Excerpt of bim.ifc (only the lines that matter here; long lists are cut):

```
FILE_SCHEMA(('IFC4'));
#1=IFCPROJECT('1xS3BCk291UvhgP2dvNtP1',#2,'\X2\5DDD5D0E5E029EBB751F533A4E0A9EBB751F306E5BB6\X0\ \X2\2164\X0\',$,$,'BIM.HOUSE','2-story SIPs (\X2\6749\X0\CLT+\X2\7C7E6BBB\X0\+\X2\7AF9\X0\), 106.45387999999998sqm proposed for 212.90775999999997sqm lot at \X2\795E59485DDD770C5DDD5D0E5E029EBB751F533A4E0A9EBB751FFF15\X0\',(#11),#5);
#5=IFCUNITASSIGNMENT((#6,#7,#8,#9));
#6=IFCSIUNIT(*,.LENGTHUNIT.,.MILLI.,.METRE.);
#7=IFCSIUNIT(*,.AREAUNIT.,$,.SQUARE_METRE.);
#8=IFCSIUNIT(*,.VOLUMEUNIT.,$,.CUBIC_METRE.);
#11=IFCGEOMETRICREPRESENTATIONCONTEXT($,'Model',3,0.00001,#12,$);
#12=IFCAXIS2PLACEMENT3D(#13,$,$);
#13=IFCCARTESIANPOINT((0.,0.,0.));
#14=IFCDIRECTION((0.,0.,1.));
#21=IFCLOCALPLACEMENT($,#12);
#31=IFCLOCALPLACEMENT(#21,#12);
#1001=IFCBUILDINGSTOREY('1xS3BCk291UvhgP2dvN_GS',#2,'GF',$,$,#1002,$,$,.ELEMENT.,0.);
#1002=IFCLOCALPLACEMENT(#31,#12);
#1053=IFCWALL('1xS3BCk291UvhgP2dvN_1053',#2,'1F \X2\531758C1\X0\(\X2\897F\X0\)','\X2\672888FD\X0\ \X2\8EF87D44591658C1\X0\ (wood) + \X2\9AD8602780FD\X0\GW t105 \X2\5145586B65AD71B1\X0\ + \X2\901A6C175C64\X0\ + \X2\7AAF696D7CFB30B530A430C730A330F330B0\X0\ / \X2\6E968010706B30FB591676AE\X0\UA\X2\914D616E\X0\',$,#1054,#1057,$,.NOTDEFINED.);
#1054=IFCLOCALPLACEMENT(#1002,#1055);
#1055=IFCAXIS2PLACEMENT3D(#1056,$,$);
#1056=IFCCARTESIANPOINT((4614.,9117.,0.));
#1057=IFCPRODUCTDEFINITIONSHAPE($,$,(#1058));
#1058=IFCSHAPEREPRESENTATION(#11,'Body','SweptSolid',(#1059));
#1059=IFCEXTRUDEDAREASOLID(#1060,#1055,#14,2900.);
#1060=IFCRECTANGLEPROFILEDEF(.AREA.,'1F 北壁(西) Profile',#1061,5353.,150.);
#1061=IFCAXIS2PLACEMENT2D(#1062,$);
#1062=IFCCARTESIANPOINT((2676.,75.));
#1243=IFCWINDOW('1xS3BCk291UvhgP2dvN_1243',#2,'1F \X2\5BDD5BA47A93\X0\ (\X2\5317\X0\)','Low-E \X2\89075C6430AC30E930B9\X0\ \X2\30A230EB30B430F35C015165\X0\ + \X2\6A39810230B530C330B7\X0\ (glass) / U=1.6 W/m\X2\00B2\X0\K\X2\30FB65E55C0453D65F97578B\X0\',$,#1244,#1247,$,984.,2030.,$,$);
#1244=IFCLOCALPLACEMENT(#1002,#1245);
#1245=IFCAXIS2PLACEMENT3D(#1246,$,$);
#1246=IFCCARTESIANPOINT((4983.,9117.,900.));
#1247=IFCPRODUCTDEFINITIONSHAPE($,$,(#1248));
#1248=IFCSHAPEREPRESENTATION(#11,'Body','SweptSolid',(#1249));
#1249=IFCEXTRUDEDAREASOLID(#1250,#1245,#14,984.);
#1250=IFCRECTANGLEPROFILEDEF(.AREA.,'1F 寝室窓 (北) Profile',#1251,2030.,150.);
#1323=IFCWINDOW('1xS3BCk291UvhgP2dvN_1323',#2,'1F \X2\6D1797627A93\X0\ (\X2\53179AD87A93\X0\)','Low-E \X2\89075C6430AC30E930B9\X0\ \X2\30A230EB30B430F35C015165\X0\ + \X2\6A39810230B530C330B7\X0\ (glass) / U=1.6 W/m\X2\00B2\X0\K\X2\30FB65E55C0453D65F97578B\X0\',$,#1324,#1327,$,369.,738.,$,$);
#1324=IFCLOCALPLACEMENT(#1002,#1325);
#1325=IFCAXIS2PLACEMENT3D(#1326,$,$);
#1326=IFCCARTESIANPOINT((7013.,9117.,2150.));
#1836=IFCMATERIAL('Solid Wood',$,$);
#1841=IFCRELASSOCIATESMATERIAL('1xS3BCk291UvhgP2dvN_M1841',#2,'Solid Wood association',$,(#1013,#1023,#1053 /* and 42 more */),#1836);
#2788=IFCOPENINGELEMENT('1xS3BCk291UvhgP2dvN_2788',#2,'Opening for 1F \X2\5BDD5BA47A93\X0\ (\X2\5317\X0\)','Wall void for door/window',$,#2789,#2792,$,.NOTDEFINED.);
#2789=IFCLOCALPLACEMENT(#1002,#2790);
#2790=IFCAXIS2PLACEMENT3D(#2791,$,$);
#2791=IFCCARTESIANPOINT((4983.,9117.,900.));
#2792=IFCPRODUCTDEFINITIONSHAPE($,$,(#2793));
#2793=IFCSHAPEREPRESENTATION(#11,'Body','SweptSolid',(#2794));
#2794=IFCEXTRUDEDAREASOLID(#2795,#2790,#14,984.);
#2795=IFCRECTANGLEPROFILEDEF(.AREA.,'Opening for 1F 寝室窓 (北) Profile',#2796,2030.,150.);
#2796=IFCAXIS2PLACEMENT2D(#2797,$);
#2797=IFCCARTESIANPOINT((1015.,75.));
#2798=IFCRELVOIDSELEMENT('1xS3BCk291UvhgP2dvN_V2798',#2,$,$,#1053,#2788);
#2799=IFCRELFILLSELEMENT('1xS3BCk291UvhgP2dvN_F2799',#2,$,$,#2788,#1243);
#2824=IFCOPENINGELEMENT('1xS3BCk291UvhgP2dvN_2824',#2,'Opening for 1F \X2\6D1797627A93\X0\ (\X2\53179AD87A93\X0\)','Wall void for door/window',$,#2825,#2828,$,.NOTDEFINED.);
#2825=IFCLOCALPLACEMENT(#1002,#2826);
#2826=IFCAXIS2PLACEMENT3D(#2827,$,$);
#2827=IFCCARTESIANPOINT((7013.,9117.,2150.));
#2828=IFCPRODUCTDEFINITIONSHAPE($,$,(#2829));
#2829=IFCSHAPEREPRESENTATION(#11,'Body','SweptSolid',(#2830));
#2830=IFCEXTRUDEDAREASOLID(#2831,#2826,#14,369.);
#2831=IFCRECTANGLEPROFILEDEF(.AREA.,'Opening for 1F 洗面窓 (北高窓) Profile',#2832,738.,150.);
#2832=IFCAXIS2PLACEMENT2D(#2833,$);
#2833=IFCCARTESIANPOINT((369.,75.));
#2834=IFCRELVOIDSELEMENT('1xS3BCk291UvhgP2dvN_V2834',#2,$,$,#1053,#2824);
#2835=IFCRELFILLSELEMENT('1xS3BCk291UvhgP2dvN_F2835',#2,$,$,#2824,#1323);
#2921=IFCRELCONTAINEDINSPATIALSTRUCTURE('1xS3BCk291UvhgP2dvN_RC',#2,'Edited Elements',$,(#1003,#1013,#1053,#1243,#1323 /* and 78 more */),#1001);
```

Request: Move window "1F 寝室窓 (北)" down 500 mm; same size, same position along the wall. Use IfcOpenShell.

```python
import numpy as np
import ifcopenshell
import ifcopenshell.api.geometry
import ifcopenshell.util.placement
import ifcopenshell.util.unit

model = ifcopenshell.open("bim.ifc")
unit_scale = ifcopenshell.util.unit.calculate_unit_scale(model)

window = model.by_guid("1xS3BCk291UvhgP2dvN_1243")
opening = window.FillsVoids[0].RelatingOpeningElement
dz = -500.0

shift = np.array([0.0, 0.0, dz])
# The window is not placed relative to its opening, so move both.
for product in (opening, window):
    matrix = ifcopenshell.util.placement.get_local_placement(product.ObjectPlacement)
    matrix[:3, 3] += shift
    ifcopenshell.api.geometry.edit_object_placement(model, product=product, matrix=matrix, is_si=False)

print(f"moved by {dz * unit_scale:+.3f} m")

model.write("bim-out.ifc")
```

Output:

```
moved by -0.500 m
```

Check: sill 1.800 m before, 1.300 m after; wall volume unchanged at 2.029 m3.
